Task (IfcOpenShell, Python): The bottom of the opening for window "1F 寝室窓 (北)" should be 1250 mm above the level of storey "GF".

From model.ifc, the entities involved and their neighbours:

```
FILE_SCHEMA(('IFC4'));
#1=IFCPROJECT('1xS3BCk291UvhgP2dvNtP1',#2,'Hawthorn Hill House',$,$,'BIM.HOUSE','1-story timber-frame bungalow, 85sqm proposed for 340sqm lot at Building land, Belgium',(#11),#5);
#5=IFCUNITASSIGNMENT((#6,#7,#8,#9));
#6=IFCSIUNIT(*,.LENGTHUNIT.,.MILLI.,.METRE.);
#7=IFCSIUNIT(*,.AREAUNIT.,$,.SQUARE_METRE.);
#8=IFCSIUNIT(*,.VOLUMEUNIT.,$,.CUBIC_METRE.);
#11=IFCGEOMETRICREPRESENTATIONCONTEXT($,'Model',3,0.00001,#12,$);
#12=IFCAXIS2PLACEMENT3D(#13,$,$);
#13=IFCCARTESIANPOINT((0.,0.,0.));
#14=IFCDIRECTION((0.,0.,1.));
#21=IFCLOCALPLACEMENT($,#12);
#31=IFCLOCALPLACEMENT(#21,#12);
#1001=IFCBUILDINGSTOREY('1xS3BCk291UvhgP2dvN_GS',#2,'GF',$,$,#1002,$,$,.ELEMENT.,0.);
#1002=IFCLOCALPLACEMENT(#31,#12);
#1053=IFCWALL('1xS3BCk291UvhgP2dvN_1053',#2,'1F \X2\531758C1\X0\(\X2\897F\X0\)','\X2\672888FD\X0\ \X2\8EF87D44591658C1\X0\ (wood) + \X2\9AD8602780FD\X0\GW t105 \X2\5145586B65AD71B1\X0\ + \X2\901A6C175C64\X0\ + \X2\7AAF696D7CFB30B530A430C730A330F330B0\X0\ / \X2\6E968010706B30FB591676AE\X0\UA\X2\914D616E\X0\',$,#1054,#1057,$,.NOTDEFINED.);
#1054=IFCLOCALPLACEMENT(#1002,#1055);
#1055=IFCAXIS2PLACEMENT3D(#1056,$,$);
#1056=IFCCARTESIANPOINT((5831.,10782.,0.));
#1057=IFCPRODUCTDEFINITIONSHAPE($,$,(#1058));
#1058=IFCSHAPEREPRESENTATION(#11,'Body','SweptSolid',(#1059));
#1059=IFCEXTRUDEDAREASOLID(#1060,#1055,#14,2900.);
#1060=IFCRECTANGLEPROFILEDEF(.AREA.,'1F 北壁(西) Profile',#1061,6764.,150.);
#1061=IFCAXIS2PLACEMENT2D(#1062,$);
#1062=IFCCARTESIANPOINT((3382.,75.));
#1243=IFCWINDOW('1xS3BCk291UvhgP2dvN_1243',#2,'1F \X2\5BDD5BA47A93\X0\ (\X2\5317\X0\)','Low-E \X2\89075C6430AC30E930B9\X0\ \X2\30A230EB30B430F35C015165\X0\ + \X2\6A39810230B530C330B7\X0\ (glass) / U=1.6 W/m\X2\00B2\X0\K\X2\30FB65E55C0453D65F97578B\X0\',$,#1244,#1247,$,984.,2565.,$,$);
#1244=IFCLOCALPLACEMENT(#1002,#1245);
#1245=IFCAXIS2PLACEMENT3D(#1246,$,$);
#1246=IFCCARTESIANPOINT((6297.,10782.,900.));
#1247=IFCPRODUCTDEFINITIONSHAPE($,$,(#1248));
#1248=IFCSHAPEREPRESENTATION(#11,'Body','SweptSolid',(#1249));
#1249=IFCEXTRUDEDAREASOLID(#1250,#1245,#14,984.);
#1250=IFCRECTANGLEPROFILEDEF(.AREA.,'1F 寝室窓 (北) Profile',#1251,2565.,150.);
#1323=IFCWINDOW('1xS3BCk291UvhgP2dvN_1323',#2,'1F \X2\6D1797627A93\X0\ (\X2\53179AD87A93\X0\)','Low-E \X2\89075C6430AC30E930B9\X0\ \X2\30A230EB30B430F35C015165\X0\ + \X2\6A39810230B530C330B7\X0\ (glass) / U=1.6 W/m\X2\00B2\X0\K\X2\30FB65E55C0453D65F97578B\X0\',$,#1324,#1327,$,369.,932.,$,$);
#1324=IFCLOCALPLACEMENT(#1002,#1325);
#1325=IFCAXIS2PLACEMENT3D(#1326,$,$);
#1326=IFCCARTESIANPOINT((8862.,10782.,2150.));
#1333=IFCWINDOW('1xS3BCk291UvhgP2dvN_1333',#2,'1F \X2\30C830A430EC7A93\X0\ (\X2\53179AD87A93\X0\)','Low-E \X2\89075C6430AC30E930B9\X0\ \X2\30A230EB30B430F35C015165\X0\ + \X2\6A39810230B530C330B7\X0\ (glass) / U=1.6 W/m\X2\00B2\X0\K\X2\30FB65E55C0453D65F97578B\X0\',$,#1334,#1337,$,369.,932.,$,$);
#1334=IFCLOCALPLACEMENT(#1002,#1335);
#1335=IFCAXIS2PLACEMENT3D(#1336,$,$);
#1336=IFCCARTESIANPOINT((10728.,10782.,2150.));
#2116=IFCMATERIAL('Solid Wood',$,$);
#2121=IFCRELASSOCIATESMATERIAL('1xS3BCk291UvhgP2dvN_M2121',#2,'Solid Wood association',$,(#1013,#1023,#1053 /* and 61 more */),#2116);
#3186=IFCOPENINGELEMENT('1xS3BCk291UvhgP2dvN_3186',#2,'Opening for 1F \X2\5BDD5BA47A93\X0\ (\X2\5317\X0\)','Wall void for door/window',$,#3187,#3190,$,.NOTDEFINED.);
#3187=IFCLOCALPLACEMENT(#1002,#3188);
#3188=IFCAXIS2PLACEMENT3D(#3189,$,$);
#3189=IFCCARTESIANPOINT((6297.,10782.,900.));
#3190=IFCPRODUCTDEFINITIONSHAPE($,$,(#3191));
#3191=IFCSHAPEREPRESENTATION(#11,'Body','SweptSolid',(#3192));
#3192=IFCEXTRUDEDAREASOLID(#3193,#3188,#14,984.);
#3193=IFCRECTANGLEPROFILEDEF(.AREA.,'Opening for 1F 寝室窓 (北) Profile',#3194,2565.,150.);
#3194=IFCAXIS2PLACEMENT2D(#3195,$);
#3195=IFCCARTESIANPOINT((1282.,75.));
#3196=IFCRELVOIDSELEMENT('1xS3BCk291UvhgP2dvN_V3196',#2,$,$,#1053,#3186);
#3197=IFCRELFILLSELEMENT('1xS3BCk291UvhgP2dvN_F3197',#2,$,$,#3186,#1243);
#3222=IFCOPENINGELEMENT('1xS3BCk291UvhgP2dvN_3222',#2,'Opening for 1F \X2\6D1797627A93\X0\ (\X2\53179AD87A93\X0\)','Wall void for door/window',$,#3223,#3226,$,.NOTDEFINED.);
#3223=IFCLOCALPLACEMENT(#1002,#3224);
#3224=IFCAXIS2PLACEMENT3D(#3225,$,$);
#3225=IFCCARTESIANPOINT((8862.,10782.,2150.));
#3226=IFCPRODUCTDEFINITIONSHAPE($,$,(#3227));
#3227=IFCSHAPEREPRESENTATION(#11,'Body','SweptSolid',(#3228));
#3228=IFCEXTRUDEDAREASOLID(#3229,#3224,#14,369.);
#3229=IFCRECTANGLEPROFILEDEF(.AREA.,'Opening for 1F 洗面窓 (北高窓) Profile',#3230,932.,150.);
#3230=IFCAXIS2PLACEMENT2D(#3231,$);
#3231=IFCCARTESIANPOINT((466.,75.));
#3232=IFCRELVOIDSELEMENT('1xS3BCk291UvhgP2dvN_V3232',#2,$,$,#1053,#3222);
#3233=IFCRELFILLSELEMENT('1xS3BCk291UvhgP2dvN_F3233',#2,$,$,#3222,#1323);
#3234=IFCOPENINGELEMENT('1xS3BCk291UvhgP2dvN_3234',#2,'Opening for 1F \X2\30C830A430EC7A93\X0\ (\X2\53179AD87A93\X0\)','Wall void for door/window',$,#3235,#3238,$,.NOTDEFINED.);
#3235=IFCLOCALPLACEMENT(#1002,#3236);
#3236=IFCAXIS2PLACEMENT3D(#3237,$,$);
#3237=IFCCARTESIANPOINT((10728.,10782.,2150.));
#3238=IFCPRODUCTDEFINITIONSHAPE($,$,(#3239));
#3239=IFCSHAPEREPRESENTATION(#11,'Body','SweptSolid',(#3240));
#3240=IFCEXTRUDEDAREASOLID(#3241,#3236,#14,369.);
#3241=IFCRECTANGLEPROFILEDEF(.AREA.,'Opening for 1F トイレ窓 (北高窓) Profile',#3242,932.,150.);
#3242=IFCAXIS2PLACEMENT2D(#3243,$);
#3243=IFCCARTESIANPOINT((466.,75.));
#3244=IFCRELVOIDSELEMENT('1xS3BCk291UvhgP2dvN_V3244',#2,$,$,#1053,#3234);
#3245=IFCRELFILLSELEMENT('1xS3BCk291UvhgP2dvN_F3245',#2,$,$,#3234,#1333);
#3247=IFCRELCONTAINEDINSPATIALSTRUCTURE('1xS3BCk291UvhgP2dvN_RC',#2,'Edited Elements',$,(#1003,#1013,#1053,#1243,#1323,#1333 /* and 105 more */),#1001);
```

```python
import numpy as np
import ifcopenshell
import ifcopenshell.api.geometry
import ifcopenshell.geom
import ifcopenshell.util.element
import ifcopenshell.util.placement
import ifcopenshell.util.shape
import ifcopenshell.util.unit

model = ifcopenshell.open("model.ifc")
unit_scale = ifcopenshell.util.unit.calculate_unit_scale(model)

window = model.by_guid("1xS3BCk291UvhgP2dvN_1243")
opening = window.FillsVoids[0].RelatingOpeningElement
storey = ifcopenshell.util.element.get_container(window, ifc_class="IfcBuildingStorey")
level = ifcopenshell.util.placement.get_local_placement(storey.ObjectPlacement)[2, 3]

# The opening's origin need not be at the sill, so measure its lowest point.
shape = ifcopenshell.geom.create_shape(ifcopenshell.geom.settings(), opening)
bottom = ifcopenshell.util.shape.get_shape_bottom_elevation(shape, shape.geometry) / unit_scale
dz = level + 1.25 / unit_scale - bottom

shift = np.array([0.0, 0.0, dz])
# The window is not placed relative to its opening, so move both.
for product in (opening, window):
    matrix = ifcopenshell.util.placement.get_local_placement(product.ObjectPlacement)
    matrix[:3, 3] += shift
    ifcopenshell.api.geometry.edit_object_placement(model, product=product, matrix=matrix, is_si=False)

print(f"moved by {dz * unit_scale:+.3f} m")

model.write("model_rev.ifc")
```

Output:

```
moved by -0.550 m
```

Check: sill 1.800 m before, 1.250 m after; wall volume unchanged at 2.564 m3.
